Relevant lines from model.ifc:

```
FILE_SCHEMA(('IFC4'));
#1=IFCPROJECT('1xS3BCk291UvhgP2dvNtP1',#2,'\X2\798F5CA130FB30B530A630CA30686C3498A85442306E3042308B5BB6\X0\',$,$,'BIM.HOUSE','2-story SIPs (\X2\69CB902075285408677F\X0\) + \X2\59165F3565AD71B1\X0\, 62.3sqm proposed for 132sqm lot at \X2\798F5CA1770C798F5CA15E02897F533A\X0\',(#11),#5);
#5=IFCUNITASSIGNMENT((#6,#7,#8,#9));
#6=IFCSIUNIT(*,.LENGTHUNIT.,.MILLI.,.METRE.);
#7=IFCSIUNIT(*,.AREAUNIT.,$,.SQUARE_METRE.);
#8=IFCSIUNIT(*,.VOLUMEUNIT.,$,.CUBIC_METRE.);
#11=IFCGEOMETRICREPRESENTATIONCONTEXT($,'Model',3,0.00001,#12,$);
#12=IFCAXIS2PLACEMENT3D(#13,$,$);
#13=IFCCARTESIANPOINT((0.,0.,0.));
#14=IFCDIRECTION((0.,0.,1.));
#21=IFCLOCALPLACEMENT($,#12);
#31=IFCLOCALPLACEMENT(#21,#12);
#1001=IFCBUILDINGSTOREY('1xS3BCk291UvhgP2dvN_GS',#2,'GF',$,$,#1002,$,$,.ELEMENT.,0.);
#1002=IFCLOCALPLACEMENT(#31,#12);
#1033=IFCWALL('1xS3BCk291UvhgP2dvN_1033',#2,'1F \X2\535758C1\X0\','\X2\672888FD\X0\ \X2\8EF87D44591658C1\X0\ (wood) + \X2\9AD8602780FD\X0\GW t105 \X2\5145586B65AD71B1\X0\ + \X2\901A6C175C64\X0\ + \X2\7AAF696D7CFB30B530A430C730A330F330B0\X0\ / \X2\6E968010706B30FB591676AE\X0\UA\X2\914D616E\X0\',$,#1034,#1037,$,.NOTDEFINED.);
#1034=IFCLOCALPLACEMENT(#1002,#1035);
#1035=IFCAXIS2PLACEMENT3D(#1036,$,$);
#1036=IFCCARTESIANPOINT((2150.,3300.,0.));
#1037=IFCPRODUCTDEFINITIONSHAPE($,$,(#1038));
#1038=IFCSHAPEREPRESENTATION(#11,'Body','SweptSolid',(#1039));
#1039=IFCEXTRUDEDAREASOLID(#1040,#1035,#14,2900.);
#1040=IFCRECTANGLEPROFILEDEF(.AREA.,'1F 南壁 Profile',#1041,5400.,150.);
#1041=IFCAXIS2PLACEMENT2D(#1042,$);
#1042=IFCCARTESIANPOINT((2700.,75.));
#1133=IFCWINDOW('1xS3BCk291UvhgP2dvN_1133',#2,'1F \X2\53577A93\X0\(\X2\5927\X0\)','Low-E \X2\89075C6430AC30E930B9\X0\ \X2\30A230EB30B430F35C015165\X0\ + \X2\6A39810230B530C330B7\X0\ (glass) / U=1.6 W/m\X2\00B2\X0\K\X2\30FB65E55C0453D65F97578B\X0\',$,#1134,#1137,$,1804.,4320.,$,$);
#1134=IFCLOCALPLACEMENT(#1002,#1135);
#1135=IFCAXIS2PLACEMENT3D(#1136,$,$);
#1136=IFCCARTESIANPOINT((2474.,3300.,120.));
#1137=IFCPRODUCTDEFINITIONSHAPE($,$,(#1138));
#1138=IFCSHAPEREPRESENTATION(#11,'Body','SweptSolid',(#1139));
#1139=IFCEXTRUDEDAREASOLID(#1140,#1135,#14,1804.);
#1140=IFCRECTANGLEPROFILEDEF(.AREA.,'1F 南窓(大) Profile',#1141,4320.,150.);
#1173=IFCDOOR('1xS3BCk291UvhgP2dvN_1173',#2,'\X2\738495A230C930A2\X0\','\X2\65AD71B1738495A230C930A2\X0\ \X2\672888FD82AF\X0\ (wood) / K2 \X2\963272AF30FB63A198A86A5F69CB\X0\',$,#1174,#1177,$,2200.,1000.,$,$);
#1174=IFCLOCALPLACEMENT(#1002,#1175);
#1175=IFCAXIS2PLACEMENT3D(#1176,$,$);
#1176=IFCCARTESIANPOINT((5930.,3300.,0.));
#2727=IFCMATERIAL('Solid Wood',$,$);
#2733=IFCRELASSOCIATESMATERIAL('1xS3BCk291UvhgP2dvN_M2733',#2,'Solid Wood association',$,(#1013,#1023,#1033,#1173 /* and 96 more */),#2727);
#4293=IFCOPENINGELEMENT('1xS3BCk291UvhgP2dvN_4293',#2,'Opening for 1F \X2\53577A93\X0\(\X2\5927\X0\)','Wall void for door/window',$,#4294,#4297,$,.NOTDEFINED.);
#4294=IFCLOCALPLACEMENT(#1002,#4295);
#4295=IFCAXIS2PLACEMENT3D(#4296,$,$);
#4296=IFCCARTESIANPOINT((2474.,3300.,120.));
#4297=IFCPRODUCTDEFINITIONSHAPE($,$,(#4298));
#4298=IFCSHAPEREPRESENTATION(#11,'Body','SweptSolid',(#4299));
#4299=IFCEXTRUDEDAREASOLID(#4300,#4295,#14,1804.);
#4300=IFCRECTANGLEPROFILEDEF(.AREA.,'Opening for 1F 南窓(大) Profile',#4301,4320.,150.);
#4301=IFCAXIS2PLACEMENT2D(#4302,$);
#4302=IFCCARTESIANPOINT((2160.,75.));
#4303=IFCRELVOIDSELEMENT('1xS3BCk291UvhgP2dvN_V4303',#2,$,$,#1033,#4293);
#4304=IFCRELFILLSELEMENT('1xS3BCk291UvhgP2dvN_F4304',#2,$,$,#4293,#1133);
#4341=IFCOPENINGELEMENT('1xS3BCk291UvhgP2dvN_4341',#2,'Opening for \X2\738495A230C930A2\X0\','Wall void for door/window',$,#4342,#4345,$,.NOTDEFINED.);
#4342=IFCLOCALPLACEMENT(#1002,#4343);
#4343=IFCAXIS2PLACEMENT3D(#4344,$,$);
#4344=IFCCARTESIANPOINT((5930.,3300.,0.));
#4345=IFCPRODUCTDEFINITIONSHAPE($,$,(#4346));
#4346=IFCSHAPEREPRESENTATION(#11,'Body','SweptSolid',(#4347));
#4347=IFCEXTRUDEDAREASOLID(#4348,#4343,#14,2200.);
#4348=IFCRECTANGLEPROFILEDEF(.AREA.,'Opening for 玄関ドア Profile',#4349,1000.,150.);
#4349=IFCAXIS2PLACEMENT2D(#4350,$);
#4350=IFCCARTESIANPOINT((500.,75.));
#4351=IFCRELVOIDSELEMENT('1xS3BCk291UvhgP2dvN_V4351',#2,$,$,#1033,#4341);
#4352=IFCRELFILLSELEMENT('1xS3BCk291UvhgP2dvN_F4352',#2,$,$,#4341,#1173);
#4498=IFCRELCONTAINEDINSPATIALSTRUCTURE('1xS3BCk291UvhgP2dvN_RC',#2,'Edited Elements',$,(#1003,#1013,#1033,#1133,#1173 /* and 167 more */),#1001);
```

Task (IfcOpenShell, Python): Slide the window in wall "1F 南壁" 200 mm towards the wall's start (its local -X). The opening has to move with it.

```python
import ifcopenshell
import ifcopenshell.api.geometry
import ifcopenshell.util.placement
import ifcopenshell.util.unit

model = ifcopenshell.open("model.ifc")
unit_scale = ifcopenshell.util.unit.calculate_unit_scale(model)

window = model.by_guid("1xS3BCk291UvhgP2dvN_1133")
opening = window.FillsVoids[0].RelatingOpeningElement
wall = opening.VoidsElements[0].RelatingBuildingElement

wall_matrix = ifcopenshell.util.placement.get_local_placement(wall.ObjectPlacement)
shift = wall_matrix[:3, 0] * -0.2 / unit_scale
before = ifcopenshell.util.placement.get_local_placement(window.ObjectPlacement)[:3, 3].copy()

# The window is not placed relative to its opening, so move both.
for product in (opening, window):
    matrix = ifcopenshell.util.placement.get_local_placement(product.ObjectPlacement)
    matrix[:3, 3] += shift
    ifcopenshell.api.geometry.edit_object_placement(model, product=product, matrix=matrix, is_si=False)

after = ifcopenshell.util.placement.get_local_placement(window.ObjectPlacement)[:3, 3]
print("window moved by", (after - before).round(3) + 0.0)

model.write("model_updated.ifc")
```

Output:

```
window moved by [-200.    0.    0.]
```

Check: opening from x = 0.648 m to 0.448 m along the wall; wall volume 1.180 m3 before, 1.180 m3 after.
